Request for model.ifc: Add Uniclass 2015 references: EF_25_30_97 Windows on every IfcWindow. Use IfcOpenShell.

First a look at what the model holds.

```python
import ifcopenshell

model = ifcopenshell.open("model.ifc")
print(model.schema)
print("classifications:", [c.Name for c in model.by_type("IfcClassification")])
for ifc_class in ("IfcDoor", "IfcRoof", "IfcStair", "IfcWall", "IfcWindow"):
    print(ifc_class, len(model.by_type(ifc_class)))
```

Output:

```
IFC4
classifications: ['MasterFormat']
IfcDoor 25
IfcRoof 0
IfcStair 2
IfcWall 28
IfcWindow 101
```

```python
import ifcopenshell
import ifcopenshell.api.classification

model = ifcopenshell.open("model.ifc")

system = ifcopenshell.api.classification.add_classification(model, classification="Uniclass 2015")

codes = {
    "IfcWindow": ("EF_25_30_97", "Windows"),
}
for ifc_class, (code, name) in codes.items():
    products = model.by_type(ifc_class)
    ifcopenshell.api.classification.add_reference(
        model, products=products, classification=system, identification=code, name=name
    )
    print(code, len(products))

model.write("model_updated.ifc")
```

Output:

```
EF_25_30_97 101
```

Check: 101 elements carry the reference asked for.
